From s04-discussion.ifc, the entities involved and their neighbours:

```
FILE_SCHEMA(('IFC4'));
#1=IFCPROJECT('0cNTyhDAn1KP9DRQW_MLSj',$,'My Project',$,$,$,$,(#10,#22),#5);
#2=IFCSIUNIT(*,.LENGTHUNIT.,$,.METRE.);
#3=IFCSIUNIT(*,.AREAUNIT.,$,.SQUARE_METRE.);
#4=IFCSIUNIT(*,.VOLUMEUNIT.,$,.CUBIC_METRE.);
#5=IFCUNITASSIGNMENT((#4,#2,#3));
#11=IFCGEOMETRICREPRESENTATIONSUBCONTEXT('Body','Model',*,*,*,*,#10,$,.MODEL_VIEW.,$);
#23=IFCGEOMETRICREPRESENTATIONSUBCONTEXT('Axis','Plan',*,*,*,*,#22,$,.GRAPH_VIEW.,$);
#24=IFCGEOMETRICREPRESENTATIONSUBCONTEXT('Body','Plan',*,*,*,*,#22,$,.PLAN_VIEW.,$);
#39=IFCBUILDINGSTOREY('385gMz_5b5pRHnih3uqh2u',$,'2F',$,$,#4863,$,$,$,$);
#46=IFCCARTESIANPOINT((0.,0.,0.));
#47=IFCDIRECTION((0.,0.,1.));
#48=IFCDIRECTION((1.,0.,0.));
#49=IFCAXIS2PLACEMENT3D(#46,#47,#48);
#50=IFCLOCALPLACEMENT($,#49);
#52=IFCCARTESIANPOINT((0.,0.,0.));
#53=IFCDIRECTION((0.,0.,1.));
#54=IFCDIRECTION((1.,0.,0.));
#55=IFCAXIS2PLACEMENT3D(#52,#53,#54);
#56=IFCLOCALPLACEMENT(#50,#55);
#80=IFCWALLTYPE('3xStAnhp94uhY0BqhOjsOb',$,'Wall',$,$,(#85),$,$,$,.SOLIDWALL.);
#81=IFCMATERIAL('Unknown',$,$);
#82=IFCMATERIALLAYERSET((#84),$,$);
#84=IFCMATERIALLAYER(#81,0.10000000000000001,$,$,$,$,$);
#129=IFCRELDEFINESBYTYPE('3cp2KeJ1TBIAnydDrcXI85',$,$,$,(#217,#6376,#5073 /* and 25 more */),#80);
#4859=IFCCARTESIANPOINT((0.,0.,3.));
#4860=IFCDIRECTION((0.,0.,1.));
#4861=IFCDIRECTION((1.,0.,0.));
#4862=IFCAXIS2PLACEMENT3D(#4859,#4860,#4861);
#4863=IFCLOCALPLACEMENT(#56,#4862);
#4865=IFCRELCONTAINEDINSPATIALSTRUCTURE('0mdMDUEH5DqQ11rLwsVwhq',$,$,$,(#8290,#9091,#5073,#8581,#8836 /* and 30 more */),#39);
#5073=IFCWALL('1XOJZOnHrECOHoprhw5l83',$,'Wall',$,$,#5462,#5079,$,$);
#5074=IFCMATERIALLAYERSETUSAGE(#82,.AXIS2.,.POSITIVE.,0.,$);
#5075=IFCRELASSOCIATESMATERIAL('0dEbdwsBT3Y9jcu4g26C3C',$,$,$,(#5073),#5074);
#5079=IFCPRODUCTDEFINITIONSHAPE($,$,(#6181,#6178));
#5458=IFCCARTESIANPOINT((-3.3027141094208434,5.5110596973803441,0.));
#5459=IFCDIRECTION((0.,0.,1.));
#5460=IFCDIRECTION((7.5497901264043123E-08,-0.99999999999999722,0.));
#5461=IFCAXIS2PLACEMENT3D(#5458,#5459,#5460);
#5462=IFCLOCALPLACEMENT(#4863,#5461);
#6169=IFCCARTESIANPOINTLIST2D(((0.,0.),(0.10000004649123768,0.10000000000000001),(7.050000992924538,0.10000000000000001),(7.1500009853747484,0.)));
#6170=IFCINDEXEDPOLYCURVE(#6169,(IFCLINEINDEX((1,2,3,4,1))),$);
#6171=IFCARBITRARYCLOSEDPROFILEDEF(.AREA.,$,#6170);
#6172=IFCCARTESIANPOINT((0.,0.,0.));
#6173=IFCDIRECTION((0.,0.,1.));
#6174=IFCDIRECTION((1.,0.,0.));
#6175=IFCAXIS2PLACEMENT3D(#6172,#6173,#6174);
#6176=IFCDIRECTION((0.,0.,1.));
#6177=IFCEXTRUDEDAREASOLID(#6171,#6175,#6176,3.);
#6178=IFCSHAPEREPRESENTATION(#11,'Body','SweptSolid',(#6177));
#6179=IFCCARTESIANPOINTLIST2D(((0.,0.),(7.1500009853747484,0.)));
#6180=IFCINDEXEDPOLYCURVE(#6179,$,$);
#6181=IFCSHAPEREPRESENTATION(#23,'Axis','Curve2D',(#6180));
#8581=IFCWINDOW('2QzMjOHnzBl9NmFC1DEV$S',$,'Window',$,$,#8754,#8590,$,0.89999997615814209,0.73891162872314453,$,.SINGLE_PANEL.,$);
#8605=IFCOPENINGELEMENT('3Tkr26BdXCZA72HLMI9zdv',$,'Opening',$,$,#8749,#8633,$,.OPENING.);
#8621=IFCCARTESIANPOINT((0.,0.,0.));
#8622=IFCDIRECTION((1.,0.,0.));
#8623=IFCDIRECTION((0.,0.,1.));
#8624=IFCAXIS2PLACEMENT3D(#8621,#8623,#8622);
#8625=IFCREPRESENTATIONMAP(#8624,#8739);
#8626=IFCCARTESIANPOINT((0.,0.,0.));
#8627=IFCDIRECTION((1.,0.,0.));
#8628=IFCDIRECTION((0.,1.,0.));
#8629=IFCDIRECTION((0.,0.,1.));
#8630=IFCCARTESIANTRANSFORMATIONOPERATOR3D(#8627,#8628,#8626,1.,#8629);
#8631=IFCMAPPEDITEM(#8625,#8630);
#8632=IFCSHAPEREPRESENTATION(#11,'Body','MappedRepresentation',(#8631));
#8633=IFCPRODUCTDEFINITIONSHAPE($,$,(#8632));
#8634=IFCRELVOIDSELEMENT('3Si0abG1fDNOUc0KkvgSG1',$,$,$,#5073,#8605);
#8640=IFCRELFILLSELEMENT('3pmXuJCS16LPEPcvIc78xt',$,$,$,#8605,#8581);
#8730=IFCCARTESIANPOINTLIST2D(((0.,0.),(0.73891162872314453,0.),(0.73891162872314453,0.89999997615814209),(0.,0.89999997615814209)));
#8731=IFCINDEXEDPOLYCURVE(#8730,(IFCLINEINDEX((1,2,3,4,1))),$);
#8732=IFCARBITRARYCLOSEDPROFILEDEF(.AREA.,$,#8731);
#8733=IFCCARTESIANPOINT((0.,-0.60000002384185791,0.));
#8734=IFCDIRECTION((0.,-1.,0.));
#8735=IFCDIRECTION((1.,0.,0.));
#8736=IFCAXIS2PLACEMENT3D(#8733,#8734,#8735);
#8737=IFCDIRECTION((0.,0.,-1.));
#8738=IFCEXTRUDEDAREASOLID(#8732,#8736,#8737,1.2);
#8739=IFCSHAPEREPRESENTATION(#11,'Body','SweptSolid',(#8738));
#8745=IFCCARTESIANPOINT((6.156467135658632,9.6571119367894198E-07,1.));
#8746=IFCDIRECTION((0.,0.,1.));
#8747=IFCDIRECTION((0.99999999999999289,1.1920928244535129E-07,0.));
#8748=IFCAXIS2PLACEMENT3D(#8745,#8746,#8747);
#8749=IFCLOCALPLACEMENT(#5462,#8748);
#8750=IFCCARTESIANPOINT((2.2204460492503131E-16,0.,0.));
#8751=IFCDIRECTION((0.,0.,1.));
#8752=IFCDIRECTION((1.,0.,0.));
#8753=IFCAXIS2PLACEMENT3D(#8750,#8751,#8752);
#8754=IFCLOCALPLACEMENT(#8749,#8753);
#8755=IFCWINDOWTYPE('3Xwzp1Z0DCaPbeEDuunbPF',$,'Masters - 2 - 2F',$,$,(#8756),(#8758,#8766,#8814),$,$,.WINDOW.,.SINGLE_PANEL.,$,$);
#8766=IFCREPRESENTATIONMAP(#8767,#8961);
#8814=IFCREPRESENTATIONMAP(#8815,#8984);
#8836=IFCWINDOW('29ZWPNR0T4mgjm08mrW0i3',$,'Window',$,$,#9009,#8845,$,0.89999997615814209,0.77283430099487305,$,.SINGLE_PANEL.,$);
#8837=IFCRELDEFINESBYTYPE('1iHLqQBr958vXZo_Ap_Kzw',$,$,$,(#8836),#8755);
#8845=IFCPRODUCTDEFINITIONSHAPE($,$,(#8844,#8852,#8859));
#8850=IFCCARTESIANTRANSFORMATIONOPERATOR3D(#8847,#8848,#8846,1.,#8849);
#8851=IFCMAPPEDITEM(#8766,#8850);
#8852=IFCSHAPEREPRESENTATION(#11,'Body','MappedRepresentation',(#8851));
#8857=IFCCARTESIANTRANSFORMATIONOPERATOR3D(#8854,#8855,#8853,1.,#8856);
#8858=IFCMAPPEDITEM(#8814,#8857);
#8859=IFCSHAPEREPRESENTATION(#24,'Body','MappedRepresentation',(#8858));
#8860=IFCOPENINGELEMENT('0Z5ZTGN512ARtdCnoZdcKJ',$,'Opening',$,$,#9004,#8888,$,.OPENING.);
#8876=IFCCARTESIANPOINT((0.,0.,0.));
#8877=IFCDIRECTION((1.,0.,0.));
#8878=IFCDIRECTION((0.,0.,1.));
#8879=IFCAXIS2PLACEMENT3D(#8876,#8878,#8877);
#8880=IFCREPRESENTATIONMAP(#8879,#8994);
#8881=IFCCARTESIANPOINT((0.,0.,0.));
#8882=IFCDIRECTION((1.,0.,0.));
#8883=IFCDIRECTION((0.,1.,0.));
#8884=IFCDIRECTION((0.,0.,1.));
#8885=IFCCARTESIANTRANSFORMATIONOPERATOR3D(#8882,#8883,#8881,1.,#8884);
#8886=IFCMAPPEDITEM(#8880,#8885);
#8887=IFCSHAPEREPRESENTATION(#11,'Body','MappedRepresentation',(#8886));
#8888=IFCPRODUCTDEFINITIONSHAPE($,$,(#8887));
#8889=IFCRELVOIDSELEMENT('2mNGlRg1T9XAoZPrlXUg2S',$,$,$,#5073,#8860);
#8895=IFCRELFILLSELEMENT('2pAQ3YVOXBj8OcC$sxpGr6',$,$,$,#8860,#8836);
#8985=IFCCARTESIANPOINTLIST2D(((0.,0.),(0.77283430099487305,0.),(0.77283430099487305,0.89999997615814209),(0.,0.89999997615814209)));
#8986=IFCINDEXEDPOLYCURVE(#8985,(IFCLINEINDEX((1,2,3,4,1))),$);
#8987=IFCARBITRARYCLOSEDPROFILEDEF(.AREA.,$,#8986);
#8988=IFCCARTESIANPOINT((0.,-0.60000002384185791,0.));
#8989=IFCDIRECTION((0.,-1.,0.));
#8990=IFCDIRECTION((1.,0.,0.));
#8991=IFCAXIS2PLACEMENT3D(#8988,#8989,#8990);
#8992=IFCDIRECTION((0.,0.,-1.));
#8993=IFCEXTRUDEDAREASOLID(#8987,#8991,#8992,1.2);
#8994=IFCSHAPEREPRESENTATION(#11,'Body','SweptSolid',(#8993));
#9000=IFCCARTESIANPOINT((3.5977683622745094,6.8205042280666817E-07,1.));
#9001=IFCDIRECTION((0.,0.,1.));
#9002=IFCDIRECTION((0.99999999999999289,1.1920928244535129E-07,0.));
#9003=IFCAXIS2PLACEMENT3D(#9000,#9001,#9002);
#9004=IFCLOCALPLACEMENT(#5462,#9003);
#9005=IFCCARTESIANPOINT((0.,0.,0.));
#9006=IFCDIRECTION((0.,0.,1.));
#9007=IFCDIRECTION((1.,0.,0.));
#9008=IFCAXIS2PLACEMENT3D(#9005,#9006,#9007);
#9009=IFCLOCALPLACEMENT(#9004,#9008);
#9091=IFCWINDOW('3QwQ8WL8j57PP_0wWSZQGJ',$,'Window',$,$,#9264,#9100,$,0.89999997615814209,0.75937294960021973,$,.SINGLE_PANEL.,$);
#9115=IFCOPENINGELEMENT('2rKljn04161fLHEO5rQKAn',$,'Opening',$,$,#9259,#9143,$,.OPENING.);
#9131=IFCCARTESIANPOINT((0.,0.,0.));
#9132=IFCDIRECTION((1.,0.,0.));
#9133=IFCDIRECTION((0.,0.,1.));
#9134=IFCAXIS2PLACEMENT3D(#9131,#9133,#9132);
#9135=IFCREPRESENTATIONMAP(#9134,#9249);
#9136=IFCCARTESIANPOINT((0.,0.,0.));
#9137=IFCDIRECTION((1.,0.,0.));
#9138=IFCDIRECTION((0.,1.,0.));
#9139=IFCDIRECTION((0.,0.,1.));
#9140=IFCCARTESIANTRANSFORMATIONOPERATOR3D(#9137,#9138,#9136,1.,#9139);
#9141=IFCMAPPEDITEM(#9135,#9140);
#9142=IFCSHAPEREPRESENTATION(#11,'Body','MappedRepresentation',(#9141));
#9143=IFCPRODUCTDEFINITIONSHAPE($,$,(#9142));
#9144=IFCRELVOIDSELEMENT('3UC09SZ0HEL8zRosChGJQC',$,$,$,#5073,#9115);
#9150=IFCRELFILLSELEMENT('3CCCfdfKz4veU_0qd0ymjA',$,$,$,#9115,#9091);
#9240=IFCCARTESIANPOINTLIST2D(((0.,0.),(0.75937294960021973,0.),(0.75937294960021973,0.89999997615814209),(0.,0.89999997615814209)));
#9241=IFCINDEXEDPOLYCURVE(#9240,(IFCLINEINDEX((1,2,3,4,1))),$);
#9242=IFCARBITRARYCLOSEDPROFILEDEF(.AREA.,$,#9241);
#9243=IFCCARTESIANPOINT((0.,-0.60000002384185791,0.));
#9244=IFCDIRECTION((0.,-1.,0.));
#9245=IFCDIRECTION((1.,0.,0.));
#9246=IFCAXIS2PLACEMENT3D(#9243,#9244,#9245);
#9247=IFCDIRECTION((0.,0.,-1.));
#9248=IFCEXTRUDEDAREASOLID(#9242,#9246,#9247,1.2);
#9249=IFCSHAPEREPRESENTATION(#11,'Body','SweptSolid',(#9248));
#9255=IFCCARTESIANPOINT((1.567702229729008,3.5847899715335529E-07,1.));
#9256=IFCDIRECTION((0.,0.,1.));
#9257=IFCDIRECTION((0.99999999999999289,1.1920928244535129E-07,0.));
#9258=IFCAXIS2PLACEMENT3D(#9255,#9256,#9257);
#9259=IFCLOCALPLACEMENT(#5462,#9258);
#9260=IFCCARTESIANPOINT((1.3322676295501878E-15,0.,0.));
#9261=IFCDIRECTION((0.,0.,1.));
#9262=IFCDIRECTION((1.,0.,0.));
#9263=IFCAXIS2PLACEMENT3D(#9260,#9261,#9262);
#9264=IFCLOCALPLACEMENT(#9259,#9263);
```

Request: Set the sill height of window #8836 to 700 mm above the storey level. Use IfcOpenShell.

```python
import numpy as np
import ifcopenshell
import ifcopenshell.api.geometry
import ifcopenshell.geom
import ifcopenshell.util.element
import ifcopenshell.util.placement
import ifcopenshell.util.shape
import ifcopenshell.util.unit

model = ifcopenshell.open("s04-discussion.ifc")
unit_scale = ifcopenshell.util.unit.calculate_unit_scale(model)

window = model.by_id(8836)
opening = window.FillsVoids[0].RelatingOpeningElement
storey = ifcopenshell.util.element.get_container(window, ifc_class="IfcBuildingStorey")
level = ifcopenshell.util.placement.get_local_placement(storey.ObjectPlacement)[2, 3]

# The opening's origin need not be at the sill, so measure its lowest point.
shape = ifcopenshell.geom.create_shape(ifcopenshell.geom.settings(), opening)
bottom = ifcopenshell.util.shape.get_shape_bottom_elevation(shape, shape.geometry) / unit_scale
dz = level + 0.7 - bottom

shift = np.array([0.0, 0.0, dz])
# The window is placed relative to its opening, so it follows when the opening moves.
matrix = ifcopenshell.util.placement.get_local_placement(opening.ObjectPlacement)
matrix[:3, 3] += shift
ifcopenshell.api.geometry.edit_object_placement(
    model, product=opening, matrix=matrix, is_si=False, should_transform_children=True
)

print(f"moved by {dz * unit_scale:+.3f} m")

model.write("s04-discussion_edited.ifc")
```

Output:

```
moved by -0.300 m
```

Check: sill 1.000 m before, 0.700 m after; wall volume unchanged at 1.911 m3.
